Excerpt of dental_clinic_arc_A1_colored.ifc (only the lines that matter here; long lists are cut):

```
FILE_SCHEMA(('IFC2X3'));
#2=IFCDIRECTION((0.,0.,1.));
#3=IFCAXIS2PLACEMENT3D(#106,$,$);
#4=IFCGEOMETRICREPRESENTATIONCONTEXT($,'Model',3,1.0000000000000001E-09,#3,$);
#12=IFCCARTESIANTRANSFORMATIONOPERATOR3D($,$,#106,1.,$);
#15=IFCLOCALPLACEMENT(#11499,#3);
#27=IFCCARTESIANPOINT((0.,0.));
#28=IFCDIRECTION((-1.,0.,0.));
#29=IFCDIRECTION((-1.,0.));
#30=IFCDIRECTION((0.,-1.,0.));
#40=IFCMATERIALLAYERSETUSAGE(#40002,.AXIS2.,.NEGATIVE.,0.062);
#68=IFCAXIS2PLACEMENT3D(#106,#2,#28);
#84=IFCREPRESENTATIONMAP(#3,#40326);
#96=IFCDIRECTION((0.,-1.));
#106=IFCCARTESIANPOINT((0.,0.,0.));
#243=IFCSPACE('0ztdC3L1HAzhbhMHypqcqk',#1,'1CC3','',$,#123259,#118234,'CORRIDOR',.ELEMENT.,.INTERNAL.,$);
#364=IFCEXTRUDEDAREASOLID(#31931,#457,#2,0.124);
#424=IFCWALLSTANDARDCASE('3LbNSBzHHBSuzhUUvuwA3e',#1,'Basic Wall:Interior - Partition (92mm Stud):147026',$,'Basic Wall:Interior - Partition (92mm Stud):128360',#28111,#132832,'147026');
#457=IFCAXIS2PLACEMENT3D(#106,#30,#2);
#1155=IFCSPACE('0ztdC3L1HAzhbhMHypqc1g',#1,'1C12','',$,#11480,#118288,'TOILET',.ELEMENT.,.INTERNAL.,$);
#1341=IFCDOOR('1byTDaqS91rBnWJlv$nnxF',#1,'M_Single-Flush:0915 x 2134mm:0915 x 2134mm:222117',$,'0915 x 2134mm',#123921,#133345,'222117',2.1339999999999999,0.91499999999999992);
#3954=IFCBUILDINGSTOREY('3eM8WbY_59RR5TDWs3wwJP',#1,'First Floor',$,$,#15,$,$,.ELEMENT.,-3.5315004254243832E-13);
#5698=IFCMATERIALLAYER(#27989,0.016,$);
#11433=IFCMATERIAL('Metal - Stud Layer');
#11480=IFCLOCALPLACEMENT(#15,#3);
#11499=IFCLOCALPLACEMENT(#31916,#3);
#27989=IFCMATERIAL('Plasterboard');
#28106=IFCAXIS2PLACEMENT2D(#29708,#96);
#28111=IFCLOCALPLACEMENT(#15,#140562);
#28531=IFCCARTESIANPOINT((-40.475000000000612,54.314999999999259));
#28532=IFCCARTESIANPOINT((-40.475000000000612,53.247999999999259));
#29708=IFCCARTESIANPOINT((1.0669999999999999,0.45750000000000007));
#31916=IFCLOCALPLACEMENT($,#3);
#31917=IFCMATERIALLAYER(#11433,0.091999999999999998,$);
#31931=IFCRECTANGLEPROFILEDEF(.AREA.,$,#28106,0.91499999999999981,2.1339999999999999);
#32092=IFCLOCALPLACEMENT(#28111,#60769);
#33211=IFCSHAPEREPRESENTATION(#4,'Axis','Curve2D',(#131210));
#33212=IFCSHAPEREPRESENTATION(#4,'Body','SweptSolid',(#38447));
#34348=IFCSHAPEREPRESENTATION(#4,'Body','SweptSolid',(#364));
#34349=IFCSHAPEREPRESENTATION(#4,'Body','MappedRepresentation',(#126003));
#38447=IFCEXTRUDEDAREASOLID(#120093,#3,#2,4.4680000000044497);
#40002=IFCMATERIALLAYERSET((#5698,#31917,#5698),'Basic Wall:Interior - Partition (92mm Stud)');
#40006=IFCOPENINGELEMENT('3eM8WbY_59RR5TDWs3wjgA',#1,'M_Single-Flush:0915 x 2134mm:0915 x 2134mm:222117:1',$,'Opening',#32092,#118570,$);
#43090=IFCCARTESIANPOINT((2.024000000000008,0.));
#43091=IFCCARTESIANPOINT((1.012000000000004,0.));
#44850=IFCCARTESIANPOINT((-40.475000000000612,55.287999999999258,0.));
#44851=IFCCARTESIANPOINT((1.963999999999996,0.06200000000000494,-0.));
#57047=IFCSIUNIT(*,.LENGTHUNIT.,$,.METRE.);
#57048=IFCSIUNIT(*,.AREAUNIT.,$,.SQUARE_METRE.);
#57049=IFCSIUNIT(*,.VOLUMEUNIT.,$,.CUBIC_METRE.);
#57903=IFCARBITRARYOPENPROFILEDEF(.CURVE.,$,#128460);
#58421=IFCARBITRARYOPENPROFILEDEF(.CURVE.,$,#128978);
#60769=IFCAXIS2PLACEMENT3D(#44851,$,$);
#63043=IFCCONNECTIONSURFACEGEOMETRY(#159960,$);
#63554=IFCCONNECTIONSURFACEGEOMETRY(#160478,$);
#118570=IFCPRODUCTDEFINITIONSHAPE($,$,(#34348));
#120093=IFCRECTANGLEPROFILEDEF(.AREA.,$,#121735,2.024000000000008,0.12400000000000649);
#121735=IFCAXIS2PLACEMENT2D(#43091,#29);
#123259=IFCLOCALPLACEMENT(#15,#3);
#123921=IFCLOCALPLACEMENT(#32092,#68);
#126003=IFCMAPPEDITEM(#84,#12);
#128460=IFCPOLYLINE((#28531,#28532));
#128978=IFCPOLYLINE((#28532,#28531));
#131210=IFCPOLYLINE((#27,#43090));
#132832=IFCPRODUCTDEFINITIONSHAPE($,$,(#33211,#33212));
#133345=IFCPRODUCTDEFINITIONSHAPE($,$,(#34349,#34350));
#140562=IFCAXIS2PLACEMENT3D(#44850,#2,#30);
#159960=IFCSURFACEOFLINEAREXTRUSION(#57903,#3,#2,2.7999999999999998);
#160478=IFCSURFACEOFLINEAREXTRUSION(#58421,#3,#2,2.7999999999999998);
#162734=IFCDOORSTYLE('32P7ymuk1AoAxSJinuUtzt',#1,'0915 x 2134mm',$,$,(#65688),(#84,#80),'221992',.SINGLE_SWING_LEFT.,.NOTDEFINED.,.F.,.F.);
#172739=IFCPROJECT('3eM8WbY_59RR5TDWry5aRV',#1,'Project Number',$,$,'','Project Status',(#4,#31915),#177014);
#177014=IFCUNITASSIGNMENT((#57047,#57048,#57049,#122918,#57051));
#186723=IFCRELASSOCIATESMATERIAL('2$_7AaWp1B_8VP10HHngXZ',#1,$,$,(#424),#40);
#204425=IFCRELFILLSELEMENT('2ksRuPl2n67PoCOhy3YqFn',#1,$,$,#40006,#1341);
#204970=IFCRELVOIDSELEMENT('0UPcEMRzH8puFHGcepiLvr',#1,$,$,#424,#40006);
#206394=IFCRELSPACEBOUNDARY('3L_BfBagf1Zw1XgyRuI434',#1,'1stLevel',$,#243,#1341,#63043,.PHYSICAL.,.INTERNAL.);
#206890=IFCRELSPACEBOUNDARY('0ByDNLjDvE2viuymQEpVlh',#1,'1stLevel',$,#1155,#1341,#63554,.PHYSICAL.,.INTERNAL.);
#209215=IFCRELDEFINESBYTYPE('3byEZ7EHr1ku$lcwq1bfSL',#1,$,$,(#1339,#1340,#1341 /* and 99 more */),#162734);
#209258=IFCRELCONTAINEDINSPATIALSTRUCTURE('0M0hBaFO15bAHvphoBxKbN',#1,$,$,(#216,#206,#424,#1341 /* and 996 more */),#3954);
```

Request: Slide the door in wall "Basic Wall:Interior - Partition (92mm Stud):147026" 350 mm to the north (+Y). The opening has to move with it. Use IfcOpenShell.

```python
import numpy as np
import ifcopenshell
import ifcopenshell.api.geometry
import ifcopenshell.util.placement
import ifcopenshell.util.unit

model = ifcopenshell.open("dental_clinic_arc_A1_colored.ifc")
unit_scale = ifcopenshell.util.unit.calculate_unit_scale(model)

door = model.by_id(1341)
opening = door.FillsVoids[0].RelatingOpeningElement
wall = opening.VoidsElements[0].RelatingBuildingElement

wall_matrix = ifcopenshell.util.placement.get_local_placement(wall.ObjectPlacement)
shift = wall_matrix[:3, 0] * -0.35 / unit_scale
before = ifcopenshell.util.placement.get_local_placement(door.ObjectPlacement)[:3, 3].copy()

# The door is placed relative to its opening, so it follows when the opening moves.
matrix = ifcopenshell.util.placement.get_local_placement(opening.ObjectPlacement)
matrix[:3, 3] += shift
ifcopenshell.api.geometry.edit_object_placement(
    model, product=opening, matrix=matrix, is_si=False, should_transform_children=True
)

# Space boundary surfaces are stored in each space's coordinates; move them too.
for rel in door.ProvidesBoundaries:
    if not rel.ConnectionGeometry:
        continue
    surface = rel.ConnectionGeometry.SurfaceOnRelatingElement
    space_matrix = ifcopenshell.util.placement.get_local_placement(rel.RelatingSpace.ObjectPlacement)
    point = np.array(surface.Position.Location.Coordinates) + space_matrix[:3, :3].T @ shift
    surface.Position = model.createIfcAxis2Placement3D(
        model.createIfcCartesianPoint(point.tolist()), surface.Position.Axis, surface.Position.RefDirection
    )

after = ifcopenshell.util.placement.get_local_placement(door.ObjectPlacement)[:3, 3]
print("door moved by", (after - before).round(3) + 0.0)

model.write("dental_clinic_arc_A1_colored-out.ifc")
```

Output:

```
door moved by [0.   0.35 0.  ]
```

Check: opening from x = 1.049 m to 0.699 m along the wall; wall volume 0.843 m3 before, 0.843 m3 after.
